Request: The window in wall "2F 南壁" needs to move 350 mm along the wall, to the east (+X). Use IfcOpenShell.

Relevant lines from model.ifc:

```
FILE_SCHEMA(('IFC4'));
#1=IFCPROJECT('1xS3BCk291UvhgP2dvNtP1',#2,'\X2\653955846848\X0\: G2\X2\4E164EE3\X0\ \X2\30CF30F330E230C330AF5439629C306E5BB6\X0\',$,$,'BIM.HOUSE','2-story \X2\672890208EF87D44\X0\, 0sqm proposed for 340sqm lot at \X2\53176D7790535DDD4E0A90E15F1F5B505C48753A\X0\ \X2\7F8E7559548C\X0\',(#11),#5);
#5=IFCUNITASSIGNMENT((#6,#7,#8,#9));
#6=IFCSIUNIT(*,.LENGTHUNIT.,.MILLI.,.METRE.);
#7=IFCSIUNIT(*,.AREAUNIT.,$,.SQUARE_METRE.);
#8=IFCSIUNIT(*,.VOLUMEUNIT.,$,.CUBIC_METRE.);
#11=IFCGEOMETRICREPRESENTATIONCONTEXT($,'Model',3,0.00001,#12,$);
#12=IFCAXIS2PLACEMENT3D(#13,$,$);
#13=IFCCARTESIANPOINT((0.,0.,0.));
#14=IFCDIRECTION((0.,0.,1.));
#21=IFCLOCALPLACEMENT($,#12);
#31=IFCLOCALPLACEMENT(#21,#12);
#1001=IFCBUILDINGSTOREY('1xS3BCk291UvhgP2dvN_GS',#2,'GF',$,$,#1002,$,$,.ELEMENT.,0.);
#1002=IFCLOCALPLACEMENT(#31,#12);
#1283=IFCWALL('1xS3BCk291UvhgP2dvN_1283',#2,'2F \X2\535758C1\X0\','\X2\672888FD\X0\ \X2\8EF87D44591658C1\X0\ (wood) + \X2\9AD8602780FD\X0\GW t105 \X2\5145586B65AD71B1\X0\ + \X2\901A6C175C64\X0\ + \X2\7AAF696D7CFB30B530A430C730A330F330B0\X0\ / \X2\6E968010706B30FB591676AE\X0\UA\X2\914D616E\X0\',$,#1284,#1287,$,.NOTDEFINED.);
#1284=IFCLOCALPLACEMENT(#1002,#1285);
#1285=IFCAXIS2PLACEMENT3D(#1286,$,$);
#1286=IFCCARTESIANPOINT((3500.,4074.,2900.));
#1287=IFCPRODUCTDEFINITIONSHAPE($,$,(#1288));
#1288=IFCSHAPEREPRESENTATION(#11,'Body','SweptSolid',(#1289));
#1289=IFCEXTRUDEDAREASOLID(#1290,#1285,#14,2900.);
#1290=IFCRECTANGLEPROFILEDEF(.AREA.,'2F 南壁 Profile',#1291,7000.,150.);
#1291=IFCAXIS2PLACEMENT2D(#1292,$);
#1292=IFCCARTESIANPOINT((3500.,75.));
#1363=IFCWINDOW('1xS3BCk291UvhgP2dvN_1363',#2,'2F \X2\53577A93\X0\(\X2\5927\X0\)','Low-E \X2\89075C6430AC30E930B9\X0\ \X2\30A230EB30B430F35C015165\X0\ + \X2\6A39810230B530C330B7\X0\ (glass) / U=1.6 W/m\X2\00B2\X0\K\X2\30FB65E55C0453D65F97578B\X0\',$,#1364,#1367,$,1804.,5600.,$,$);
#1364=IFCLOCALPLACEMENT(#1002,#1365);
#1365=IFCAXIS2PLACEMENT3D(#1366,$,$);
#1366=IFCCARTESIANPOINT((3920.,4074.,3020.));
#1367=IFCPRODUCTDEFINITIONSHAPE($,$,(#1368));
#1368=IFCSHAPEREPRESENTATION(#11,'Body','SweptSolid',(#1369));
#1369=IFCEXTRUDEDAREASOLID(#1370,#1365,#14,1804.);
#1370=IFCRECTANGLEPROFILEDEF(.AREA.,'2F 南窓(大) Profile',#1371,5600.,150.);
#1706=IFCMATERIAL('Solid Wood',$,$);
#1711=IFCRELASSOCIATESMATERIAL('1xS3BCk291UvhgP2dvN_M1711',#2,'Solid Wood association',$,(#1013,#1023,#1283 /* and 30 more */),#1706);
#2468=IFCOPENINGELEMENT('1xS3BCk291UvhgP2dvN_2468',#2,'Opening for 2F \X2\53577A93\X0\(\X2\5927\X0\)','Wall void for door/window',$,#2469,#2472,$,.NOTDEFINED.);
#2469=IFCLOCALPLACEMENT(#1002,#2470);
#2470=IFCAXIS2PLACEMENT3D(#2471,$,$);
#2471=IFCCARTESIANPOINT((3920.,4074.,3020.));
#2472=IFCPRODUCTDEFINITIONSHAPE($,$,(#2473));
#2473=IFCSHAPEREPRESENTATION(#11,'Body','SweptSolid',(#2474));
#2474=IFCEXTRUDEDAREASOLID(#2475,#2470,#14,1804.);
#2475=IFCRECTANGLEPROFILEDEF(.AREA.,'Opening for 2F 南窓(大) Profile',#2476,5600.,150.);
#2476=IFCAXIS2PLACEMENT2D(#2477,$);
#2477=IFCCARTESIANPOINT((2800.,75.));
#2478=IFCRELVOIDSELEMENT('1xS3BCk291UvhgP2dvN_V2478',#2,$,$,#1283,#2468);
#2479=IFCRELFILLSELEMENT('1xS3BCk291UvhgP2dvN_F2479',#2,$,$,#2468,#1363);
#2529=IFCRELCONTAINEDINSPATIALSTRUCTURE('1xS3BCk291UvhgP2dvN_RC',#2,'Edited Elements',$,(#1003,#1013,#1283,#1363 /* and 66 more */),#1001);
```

```python
import ifcopenshell
import ifcopenshell.api.geometry
import ifcopenshell.util.placement
import ifcopenshell.util.unit

model = ifcopenshell.open("model.ifc")
unit_scale = ifcopenshell.util.unit.calculate_unit_scale(model)

window = model.by_id(1363)
opening = window.FillsVoids[0].RelatingOpeningElement
wall = opening.VoidsElements[0].RelatingBuildingElement

wall_matrix = ifcopenshell.util.placement.get_local_placement(wall.ObjectPlacement)
shift = wall_matrix[:3, 0] * 0.35 / unit_scale
before = ifcopenshell.util.placement.get_local_placement(window.ObjectPlacement)[:3, 3].copy()

# The window is not placed relative to its opening, so move both.
for product in (opening, window):
    matrix = ifcopenshell.util.placement.get_local_placement(product.ObjectPlacement)
    matrix[:3, 3] += shift
    ifcopenshell.api.geometry.edit_object_placement(model, product=product, matrix=matrix, is_si=False)

after = ifcopenshell.util.placement.get_local_placement(window.ObjectPlacement)[:3, 3]
print("window moved by", (after - before).round(3) + 0.0)

model.write("model_rev.ifc")
```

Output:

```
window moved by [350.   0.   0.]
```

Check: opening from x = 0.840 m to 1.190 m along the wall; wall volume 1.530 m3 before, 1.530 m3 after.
